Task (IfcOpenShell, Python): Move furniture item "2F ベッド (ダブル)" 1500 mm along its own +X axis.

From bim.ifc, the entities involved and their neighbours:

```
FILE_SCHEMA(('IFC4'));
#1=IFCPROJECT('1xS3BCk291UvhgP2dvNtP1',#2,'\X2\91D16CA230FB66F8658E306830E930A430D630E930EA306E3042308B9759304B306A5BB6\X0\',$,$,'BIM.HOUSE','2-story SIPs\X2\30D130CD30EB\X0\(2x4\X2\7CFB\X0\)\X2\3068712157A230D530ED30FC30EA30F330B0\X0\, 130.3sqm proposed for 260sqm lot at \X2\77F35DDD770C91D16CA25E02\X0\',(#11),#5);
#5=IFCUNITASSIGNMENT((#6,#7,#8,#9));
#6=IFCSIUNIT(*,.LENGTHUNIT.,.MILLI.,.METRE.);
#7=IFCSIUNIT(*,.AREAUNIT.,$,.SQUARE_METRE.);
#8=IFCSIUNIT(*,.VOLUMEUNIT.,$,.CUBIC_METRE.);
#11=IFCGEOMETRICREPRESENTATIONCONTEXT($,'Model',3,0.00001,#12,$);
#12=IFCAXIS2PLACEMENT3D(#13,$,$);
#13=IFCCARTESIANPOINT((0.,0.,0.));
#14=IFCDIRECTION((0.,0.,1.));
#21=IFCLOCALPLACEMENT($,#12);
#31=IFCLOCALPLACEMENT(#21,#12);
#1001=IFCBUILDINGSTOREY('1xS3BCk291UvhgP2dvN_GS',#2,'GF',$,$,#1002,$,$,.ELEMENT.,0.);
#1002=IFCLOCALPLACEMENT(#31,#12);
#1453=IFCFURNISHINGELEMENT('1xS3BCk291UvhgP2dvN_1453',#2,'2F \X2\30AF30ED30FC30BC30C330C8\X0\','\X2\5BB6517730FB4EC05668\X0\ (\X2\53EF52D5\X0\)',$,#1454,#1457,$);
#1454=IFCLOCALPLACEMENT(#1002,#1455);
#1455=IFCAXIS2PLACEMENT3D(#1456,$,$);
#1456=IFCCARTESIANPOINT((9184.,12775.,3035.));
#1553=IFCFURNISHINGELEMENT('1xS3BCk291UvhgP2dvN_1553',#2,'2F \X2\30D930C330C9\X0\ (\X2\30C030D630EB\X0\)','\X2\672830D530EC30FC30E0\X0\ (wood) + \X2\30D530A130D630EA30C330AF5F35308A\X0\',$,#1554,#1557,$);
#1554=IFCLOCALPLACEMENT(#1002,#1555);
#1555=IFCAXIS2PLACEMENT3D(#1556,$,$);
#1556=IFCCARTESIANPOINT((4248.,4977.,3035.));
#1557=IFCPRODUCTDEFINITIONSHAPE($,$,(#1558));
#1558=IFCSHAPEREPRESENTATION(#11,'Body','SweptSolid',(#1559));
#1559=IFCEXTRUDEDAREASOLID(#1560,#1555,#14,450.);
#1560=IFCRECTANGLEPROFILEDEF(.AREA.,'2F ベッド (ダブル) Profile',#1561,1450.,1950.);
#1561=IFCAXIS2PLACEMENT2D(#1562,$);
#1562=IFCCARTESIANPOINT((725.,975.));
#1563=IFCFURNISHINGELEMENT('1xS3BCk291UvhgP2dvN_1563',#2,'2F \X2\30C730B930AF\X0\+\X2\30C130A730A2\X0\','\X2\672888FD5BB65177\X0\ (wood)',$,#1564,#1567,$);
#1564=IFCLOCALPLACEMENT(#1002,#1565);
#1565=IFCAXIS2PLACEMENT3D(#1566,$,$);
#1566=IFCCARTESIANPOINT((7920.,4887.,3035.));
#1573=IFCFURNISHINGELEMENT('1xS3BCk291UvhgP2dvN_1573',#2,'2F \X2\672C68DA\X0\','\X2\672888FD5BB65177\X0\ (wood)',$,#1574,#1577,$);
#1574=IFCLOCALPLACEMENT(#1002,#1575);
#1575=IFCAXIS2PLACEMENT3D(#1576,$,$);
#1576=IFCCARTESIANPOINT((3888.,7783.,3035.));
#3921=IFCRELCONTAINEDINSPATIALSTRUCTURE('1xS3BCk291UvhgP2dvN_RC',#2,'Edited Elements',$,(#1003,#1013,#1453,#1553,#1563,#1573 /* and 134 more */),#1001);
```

```python
import ifcopenshell
import ifcopenshell.api.geometry
import ifcopenshell.util.placement
import ifcopenshell.util.unit

model = ifcopenshell.open("bim.ifc")
unit_scale = ifcopenshell.util.unit.calculate_unit_scale(model)

item = model.by_id(1553)
matrix = ifcopenshell.util.placement.get_local_placement(item.ObjectPlacement)
matrix[:3, 3] += matrix[:3, 0] * 1.5 / unit_scale
ifcopenshell.api.geometry.edit_object_placement(model, product=item, matrix=matrix, is_si=False)

print(ifcopenshell.util.placement.get_local_placement(item.ObjectPlacement).round(3) + 0.0)

model.write("bim-out.ifc")
```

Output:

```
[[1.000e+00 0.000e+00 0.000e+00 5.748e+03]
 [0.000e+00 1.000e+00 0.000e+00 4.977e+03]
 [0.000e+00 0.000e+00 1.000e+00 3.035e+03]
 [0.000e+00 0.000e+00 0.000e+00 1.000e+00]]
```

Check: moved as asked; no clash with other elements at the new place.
